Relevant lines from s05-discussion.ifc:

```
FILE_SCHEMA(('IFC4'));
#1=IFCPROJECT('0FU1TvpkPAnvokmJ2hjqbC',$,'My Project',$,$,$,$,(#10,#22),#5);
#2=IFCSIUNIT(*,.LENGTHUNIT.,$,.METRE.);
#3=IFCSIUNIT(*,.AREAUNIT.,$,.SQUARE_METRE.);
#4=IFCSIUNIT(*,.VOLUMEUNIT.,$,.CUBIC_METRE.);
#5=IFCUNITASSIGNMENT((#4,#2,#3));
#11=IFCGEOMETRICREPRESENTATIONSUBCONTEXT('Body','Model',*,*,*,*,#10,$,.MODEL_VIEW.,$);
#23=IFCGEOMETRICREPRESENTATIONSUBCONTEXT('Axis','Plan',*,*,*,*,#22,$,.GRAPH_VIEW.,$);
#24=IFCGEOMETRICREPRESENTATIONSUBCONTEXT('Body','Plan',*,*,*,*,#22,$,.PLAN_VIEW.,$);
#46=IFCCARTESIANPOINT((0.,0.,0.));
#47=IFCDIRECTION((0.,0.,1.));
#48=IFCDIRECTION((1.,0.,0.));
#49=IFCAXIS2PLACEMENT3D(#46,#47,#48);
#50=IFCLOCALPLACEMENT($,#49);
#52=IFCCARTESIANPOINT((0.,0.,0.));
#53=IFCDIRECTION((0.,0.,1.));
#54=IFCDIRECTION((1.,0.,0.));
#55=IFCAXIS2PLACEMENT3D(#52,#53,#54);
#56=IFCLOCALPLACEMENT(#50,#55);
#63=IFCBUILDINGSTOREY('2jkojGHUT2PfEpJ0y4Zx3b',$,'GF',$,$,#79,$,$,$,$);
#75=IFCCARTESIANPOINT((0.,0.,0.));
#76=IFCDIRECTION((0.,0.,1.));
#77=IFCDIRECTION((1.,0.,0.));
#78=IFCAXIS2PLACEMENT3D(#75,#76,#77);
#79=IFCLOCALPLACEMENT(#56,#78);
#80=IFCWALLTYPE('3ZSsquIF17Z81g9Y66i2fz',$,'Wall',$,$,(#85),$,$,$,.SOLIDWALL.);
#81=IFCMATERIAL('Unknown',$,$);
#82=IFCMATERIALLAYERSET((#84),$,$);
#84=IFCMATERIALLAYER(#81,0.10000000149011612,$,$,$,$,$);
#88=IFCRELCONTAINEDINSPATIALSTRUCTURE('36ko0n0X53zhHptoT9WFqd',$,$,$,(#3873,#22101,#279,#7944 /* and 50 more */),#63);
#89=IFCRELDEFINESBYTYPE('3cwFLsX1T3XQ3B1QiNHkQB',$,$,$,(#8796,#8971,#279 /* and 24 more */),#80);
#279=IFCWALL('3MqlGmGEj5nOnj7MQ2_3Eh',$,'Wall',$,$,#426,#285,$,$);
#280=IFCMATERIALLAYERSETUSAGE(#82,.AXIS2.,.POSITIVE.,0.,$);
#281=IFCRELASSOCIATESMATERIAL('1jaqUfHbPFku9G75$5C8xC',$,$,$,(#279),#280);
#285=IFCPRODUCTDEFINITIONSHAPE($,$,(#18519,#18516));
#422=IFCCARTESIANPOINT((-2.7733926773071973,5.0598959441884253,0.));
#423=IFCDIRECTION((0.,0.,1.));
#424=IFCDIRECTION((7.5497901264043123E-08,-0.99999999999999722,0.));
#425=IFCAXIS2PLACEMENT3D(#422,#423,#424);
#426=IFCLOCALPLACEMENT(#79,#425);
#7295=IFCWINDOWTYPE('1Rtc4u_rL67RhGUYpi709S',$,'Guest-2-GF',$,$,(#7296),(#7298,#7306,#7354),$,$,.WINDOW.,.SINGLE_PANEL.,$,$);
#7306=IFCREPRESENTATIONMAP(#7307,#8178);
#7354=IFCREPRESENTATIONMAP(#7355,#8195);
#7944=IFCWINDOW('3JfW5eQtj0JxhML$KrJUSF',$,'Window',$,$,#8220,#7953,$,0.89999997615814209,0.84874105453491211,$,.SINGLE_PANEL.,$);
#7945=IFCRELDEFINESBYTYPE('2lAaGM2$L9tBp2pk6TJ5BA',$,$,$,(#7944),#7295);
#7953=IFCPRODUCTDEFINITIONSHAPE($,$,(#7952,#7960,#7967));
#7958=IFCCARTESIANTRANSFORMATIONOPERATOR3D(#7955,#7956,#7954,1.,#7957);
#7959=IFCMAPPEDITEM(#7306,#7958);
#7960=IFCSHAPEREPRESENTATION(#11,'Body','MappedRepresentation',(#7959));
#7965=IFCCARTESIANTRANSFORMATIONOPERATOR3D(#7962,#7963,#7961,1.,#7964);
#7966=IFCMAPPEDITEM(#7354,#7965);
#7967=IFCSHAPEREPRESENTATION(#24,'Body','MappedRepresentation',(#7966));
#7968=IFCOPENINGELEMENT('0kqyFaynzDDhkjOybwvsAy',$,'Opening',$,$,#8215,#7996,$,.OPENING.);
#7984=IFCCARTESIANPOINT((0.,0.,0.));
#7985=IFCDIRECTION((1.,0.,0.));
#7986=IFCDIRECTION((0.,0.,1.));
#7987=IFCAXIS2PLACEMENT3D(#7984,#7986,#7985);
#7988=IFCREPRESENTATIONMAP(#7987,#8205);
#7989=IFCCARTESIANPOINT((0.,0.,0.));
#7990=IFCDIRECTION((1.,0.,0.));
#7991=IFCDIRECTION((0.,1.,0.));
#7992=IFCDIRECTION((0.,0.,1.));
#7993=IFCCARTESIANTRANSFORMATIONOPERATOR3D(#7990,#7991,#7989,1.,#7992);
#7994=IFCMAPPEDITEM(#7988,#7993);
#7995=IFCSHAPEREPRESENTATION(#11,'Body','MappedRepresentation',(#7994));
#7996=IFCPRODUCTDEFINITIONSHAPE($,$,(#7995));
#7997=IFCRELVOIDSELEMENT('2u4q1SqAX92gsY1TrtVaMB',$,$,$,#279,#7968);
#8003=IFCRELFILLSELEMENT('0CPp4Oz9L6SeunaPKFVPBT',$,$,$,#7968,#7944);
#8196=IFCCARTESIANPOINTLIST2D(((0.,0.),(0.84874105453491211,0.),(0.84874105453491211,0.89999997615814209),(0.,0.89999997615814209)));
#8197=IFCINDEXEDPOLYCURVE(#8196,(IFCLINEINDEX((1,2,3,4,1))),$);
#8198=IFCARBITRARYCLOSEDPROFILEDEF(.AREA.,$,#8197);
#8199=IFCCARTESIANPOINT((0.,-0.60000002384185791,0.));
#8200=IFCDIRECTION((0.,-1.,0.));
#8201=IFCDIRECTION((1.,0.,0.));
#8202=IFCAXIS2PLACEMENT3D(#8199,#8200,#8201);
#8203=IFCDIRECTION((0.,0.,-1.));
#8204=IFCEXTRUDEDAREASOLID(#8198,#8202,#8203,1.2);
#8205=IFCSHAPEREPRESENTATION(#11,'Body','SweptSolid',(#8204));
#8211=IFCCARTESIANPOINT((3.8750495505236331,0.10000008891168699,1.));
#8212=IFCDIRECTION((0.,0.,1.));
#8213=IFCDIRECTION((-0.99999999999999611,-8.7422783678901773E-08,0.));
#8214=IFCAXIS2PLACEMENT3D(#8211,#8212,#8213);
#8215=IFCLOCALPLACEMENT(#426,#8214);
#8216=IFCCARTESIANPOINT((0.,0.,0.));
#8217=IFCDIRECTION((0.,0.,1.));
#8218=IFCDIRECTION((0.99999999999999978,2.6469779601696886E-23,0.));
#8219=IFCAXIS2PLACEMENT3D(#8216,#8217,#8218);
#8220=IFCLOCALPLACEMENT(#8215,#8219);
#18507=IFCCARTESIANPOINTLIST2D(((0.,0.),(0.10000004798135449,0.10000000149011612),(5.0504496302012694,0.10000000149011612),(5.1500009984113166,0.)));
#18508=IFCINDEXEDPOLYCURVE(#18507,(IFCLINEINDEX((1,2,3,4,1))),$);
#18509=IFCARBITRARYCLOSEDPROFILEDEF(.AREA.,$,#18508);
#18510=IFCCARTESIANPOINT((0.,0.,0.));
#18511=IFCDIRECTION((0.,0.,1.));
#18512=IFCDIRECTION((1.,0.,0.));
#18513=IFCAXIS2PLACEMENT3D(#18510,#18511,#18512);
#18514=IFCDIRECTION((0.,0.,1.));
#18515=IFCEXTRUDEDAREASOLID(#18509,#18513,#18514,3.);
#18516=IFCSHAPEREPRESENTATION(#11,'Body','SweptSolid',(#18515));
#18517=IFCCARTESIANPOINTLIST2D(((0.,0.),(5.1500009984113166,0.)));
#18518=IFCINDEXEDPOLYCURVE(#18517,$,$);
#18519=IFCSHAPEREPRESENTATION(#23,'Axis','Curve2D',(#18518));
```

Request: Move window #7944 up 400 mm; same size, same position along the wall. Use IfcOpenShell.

```python
import numpy as np
import ifcopenshell
import ifcopenshell.api.geometry
import ifcopenshell.util.placement
import ifcopenshell.util.unit

model = ifcopenshell.open("s05-discussion.ifc")
unit_scale = ifcopenshell.util.unit.calculate_unit_scale(model)

window = model.by_id(7944)
opening = window.FillsVoids[0].RelatingOpeningElement
dz = 0.4 / unit_scale

shift = np.array([0.0, 0.0, dz])
# The window is placed relative to its opening, so it follows when the opening moves.
matrix = ifcopenshell.util.placement.get_local_placement(opening.ObjectPlacement)
matrix[:3, 3] += shift
ifcopenshell.api.geometry.edit_object_placement(
    model, product=opening, matrix=matrix, is_si=False, should_transform_children=True
)

print(f"moved by {dz * unit_scale:+.3f} m")

model.write("s05-discussion_rev.ifc")
```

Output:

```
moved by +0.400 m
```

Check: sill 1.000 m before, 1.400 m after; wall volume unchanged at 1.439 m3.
